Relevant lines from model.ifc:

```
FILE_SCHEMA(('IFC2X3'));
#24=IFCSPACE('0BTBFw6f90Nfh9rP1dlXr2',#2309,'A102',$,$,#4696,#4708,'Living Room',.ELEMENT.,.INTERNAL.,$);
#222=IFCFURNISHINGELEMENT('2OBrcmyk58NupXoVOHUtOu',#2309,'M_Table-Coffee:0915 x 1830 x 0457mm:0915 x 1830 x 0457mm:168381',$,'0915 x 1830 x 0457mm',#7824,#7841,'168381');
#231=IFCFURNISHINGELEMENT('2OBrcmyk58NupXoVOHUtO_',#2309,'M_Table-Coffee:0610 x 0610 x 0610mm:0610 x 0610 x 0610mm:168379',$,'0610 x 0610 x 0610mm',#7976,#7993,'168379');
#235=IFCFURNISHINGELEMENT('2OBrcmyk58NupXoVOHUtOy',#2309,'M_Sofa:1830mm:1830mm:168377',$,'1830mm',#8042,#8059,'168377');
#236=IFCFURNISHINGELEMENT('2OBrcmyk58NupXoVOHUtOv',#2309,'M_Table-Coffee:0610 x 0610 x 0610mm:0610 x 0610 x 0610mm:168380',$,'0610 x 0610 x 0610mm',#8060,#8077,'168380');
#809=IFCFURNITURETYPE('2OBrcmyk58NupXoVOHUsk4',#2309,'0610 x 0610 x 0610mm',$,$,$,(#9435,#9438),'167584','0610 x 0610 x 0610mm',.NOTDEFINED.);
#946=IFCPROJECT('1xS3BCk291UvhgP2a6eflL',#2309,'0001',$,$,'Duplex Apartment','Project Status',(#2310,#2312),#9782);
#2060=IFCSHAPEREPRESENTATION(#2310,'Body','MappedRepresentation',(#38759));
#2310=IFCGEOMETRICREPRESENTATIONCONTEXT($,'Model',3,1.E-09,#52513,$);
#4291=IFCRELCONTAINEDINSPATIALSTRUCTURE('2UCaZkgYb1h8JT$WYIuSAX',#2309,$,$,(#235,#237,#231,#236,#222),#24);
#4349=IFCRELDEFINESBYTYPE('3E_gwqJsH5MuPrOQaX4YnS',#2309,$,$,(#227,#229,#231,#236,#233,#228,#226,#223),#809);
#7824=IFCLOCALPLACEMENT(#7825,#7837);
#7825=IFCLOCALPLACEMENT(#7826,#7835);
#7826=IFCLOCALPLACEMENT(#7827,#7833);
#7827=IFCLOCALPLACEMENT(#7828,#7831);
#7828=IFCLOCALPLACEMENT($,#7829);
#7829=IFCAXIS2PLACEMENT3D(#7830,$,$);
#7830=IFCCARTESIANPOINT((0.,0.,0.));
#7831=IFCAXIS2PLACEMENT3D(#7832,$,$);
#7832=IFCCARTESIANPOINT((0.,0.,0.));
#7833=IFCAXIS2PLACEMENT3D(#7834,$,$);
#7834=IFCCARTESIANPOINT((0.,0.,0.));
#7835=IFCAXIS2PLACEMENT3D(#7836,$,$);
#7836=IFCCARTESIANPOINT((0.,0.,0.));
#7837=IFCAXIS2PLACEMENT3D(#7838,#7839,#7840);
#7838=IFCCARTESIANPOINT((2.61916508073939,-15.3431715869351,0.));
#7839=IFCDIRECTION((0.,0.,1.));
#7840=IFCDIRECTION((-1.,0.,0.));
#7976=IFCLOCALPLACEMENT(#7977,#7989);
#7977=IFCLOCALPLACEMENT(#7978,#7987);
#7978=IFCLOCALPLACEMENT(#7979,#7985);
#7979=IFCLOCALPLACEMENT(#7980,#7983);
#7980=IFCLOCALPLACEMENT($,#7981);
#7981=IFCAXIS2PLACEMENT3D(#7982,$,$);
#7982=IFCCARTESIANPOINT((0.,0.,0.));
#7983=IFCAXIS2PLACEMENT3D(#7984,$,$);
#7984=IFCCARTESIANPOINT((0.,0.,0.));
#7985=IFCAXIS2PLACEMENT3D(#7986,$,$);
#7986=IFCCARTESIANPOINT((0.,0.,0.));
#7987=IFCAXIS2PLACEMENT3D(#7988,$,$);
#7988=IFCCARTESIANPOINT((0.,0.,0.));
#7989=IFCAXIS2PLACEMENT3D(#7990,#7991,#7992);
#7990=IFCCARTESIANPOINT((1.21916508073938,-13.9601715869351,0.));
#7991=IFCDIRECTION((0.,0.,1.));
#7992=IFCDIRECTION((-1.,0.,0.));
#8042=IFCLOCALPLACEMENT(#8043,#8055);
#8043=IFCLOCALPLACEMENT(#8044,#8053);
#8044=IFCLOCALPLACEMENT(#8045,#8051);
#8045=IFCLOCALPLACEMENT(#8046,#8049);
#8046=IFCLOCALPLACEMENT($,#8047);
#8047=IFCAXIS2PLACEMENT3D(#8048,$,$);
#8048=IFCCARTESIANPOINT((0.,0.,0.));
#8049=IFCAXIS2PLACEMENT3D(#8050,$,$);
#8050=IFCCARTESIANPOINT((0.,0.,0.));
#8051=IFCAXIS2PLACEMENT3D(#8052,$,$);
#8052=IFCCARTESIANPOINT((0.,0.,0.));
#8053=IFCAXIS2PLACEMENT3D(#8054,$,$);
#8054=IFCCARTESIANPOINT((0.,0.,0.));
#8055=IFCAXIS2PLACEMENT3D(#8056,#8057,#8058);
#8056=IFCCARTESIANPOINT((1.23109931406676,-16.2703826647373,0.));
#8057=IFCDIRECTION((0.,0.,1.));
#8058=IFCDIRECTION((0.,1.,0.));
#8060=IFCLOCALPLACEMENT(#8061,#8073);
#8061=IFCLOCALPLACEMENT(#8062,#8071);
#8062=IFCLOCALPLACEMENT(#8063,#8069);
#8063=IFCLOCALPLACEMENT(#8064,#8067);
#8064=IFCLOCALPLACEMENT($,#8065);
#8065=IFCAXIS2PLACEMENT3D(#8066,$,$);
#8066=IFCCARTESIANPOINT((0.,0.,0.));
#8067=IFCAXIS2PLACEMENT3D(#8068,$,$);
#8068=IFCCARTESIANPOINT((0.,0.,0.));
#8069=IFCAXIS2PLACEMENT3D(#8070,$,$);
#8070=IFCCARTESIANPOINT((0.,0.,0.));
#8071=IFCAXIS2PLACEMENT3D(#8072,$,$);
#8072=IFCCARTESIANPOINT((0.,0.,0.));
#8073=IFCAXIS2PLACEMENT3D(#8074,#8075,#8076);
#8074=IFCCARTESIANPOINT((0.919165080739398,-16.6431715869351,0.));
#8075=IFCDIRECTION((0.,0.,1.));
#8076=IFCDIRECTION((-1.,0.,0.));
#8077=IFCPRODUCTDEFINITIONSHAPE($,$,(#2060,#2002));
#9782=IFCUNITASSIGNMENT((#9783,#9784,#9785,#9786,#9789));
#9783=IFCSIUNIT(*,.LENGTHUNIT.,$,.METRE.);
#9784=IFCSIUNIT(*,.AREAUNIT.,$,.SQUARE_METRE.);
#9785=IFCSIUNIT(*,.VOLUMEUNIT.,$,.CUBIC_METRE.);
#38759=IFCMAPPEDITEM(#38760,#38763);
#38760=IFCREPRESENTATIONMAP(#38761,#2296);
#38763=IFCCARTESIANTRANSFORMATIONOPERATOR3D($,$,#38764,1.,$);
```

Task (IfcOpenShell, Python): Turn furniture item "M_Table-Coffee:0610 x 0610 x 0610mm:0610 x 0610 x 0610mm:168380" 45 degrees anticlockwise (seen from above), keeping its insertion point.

```python
import ifcopenshell
import ifcopenshell.api.geometry
import ifcopenshell.util.placement

model = ifcopenshell.open("model.ifc")

item = model.by_guid("2OBrcmyk58NupXoVOHUtOv")
matrix = ifcopenshell.util.placement.get_local_placement(item.ObjectPlacement)
matrix = matrix @ ifcopenshell.util.placement.rotation(45, "Z")
ifcopenshell.api.geometry.edit_object_placement(model, product=item, matrix=matrix, is_si=False)

print(ifcopenshell.util.placement.get_local_placement(item.ObjectPlacement).round(3) + 0.0)

model.write("model_edited.ifc")
```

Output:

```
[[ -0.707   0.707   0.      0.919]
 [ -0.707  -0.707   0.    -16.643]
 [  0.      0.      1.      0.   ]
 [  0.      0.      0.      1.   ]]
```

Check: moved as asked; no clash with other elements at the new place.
